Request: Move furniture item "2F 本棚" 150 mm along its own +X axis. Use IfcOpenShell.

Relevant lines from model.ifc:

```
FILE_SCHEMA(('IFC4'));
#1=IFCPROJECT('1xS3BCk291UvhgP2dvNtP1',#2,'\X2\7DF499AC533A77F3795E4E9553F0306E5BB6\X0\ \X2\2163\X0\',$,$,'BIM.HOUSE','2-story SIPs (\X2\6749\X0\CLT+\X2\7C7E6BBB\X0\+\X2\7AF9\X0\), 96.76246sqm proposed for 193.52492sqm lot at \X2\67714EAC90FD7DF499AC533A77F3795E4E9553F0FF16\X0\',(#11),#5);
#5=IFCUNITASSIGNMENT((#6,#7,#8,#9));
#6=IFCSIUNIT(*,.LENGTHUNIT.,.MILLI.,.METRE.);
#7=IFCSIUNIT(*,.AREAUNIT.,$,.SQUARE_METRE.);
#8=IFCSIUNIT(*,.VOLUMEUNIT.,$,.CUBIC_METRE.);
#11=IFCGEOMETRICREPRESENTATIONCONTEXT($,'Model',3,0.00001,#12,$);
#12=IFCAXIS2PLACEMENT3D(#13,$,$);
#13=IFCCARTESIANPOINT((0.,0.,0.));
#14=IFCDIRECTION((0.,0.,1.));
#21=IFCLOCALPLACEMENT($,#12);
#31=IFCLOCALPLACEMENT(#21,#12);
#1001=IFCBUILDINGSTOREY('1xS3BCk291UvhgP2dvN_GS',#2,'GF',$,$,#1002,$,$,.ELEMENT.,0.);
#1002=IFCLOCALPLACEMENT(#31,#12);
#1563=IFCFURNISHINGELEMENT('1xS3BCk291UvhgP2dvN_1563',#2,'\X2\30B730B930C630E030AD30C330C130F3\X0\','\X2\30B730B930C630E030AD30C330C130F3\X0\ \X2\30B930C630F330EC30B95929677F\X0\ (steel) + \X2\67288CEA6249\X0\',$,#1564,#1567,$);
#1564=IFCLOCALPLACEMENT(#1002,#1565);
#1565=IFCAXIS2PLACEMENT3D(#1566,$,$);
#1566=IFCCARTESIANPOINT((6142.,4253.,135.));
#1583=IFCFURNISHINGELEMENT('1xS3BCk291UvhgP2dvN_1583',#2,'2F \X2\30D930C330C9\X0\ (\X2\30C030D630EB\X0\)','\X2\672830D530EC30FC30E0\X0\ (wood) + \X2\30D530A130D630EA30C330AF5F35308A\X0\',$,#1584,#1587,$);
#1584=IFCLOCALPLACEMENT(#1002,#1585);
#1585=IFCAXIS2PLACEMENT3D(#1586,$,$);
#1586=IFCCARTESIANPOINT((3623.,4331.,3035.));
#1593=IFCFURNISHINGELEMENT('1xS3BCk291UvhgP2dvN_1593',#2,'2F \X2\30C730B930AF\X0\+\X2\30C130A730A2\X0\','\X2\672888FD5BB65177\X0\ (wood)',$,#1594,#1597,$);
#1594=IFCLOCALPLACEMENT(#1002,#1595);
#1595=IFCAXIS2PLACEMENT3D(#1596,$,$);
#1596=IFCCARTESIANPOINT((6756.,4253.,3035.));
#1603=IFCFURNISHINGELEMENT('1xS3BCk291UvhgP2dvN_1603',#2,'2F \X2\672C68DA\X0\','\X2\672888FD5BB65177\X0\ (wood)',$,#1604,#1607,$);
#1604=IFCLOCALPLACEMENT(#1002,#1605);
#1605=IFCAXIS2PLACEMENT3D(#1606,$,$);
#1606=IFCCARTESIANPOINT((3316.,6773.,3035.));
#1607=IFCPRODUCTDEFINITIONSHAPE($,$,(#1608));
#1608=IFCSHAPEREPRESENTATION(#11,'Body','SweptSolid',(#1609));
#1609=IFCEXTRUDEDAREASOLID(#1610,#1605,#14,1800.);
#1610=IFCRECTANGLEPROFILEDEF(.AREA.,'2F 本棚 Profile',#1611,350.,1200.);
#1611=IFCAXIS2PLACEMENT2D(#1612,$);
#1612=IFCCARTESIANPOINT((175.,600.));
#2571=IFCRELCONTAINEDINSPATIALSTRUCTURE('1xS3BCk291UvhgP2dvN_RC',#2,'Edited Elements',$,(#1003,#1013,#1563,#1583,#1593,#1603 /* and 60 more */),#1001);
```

```python
import ifcopenshell
import ifcopenshell.api.geometry
import ifcopenshell.util.placement
import ifcopenshell.util.unit

model = ifcopenshell.open("model.ifc")
unit_scale = ifcopenshell.util.unit.calculate_unit_scale(model)

item = model.by_id(1603)
matrix = ifcopenshell.util.placement.get_local_placement(item.ObjectPlacement)
matrix[:3, 3] += matrix[:3, 0] * 0.15 / unit_scale
ifcopenshell.api.geometry.edit_object_placement(model, product=item, matrix=matrix, is_si=False)

print(ifcopenshell.util.placement.get_local_placement(item.ObjectPlacement).round(3) + 0.0)

model.write("model_rev.ifc")
```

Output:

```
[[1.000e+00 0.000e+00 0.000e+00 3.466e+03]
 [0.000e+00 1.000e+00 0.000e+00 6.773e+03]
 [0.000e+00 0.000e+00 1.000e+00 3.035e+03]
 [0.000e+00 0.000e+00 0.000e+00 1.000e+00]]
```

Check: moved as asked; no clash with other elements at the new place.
